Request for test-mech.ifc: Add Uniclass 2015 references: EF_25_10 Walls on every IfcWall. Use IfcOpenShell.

First a look at what the model holds.

```python
import ifcopenshell

model = ifcopenshell.open("test-mech.ifc")
print(model.schema)
print("classifications:", [c.Name for c in model.by_type("IfcClassification")])
for ifc_class in ("IfcDoor", "IfcRoof", "IfcStair", "IfcWall", "IfcWindow"):
    print(ifc_class, len(model.by_type(ifc_class)))
```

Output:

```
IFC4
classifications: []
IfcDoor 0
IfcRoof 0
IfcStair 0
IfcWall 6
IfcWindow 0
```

```python
import ifcopenshell
import ifcopenshell.api.classification

model = ifcopenshell.open("test-mech.ifc")

system = ifcopenshell.api.classification.add_classification(model, classification="Uniclass 2015")

codes = {
    "IfcWall": ("EF_25_10", "Walls"),
}
for ifc_class, (code, name) in codes.items():
    products = model.by_type(ifc_class)
    ifcopenshell.api.classification.add_reference(
        model, products=products, classification=system, identification=code, name=name
    )
    print(code, len(products))

model.write("test-mech_rev.ifc")
```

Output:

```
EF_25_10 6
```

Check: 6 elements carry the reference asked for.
